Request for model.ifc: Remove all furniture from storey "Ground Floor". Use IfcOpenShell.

First a look at what the model holds.

```python
import ifcopenshell
import ifcopenshell.util.element

model = ifcopenshell.open("model.ifc")
print(model.schema)
storey = next(s for s in model.by_type("IfcBuildingStorey") if s.Name == "Ground Floor")
furniture = [e for e in ifcopenshell.util.element.get_decomposition(storey) if e.is_a("IfcFurnishingElement")]
seen = {}
for e in furniture:
    element_type = ifcopenshell.util.element.get_type(e)
    name = element_type.Name if element_type not in (None, e) else None
    seen[name] = seen.get(name, 0) + 1
for name, count in sorted(seen.items(), key=str):
    print(count, "x", name)
```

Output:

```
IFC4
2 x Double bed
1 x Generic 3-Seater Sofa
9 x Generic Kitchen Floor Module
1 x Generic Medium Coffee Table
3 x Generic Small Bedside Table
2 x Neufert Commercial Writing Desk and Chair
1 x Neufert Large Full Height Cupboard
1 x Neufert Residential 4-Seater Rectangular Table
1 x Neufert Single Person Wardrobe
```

```python
import ifcopenshell
import ifcopenshell.api.root
import ifcopenshell.util.element

model = ifcopenshell.open("model.ifc")

storey = next(s for s in model.by_type("IfcBuildingStorey") if s.Name == "Ground Floor")
furniture = [e for e in ifcopenshell.util.element.get_decomposition(storey) if e.is_a("IfcFurnishingElement")]

for e in furniture:
    ifcopenshell.api.root.remove_product(model, product=e)
print(len(furniture), "removed")

model.write("model_edited.ifc")
```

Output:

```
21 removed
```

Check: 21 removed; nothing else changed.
